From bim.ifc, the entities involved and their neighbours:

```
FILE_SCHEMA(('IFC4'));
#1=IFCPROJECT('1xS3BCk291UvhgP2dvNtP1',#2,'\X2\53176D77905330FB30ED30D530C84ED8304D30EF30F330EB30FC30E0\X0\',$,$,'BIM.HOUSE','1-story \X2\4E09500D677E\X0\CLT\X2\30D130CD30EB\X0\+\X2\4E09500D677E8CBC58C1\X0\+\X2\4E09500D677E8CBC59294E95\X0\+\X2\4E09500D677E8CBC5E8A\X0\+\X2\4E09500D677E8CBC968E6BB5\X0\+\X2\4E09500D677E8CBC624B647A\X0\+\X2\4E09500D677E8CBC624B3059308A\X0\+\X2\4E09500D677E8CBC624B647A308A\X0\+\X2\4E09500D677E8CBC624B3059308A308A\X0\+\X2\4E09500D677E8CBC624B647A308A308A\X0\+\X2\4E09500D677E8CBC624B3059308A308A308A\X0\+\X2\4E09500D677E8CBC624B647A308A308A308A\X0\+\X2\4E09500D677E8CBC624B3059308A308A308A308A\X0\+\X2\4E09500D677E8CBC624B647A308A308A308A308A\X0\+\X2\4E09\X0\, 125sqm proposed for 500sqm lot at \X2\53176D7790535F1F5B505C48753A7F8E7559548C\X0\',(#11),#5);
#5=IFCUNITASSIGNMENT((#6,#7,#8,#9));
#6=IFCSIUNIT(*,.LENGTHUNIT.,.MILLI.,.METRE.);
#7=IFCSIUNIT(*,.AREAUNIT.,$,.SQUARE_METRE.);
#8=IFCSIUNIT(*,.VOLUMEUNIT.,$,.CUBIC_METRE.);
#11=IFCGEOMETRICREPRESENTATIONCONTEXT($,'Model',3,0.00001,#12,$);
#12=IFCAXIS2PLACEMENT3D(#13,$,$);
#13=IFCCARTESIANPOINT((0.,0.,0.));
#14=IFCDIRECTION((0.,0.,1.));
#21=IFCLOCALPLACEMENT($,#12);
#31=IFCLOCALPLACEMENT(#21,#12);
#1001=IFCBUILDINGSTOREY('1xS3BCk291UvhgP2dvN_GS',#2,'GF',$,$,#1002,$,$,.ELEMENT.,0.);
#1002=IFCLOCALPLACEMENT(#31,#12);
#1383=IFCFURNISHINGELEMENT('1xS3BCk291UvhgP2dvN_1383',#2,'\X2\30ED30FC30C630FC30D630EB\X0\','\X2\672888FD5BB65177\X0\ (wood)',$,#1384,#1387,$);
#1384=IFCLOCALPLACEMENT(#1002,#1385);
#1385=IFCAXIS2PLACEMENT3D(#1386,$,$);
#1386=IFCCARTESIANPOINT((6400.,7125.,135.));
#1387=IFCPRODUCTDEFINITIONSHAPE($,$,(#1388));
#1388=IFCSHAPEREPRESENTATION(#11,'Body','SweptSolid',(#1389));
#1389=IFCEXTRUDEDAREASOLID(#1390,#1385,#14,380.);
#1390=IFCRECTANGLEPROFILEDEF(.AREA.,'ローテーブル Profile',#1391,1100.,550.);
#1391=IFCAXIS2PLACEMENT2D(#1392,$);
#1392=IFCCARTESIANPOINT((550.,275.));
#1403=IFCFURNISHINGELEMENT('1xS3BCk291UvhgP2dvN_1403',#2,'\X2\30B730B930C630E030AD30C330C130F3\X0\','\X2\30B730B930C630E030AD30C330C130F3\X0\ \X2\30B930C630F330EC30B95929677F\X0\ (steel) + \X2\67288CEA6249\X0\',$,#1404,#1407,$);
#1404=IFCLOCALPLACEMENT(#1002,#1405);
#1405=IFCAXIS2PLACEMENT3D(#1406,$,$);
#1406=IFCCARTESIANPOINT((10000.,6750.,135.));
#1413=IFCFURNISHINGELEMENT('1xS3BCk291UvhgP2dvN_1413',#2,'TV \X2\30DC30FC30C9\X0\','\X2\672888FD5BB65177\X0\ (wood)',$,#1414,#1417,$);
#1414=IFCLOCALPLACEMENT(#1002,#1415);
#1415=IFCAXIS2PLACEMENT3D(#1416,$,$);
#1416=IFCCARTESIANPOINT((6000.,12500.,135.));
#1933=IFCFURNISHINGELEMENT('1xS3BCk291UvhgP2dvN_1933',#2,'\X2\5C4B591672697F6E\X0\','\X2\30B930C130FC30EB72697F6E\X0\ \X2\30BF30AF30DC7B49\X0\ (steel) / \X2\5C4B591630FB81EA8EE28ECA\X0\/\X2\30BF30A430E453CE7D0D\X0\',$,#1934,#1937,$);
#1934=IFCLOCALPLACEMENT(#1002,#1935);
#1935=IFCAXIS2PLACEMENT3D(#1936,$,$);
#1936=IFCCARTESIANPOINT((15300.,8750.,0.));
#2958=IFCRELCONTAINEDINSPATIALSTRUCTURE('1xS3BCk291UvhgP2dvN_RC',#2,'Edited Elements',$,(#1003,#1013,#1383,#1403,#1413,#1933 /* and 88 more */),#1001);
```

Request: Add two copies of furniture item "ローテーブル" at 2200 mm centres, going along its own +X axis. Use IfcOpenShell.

```python
import ifcopenshell
import ifcopenshell.api.geometry
import ifcopenshell.api.root
import ifcopenshell.util.element
import ifcopenshell.util.placement

model = ifcopenshell.open("bim.ifc")


def reuse_history(source, copy):
    """copy_class also copies each property set's owner history, people and application; keep the originals."""
    for rel in copy.IsDefinedBy:
        if rel.is_a("IfcRelDefinesByProperties") and (history := rel.RelatingPropertyDefinition.OwnerHistory):
            rel.RelatingPropertyDefinition.OwnerHistory = source.OwnerHistory
            ifcopenshell.util.element.remove_deep2(model, history)


source = model.by_guid("1xS3BCk291UvhgP2dvN_1383")
base = ifcopenshell.util.placement.get_local_placement(source.ObjectPlacement)
step = base[:3, 0] * 2200.0

for i in range(1, 3):
    copy = ifcopenshell.api.root.copy_class(model, product=source)
    copy.Representation = ifcopenshell.util.element.copy_deep(
        model, source.Representation, exclude=["IfcGeometricRepresentationContext", "IfcRepresentationMap"]
    )
    reuse_history(source, copy)
    matrix = base.copy()
    matrix[:3, 3] += i * step
    print("added at", matrix[:3, 3].round(3) + 0.0)
    ifcopenshell.api.geometry.edit_object_placement(model, product=copy, matrix=matrix, is_si=False)

model.write("bim-out.ifc")
```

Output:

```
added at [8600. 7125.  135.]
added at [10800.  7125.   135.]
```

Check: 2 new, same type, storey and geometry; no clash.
